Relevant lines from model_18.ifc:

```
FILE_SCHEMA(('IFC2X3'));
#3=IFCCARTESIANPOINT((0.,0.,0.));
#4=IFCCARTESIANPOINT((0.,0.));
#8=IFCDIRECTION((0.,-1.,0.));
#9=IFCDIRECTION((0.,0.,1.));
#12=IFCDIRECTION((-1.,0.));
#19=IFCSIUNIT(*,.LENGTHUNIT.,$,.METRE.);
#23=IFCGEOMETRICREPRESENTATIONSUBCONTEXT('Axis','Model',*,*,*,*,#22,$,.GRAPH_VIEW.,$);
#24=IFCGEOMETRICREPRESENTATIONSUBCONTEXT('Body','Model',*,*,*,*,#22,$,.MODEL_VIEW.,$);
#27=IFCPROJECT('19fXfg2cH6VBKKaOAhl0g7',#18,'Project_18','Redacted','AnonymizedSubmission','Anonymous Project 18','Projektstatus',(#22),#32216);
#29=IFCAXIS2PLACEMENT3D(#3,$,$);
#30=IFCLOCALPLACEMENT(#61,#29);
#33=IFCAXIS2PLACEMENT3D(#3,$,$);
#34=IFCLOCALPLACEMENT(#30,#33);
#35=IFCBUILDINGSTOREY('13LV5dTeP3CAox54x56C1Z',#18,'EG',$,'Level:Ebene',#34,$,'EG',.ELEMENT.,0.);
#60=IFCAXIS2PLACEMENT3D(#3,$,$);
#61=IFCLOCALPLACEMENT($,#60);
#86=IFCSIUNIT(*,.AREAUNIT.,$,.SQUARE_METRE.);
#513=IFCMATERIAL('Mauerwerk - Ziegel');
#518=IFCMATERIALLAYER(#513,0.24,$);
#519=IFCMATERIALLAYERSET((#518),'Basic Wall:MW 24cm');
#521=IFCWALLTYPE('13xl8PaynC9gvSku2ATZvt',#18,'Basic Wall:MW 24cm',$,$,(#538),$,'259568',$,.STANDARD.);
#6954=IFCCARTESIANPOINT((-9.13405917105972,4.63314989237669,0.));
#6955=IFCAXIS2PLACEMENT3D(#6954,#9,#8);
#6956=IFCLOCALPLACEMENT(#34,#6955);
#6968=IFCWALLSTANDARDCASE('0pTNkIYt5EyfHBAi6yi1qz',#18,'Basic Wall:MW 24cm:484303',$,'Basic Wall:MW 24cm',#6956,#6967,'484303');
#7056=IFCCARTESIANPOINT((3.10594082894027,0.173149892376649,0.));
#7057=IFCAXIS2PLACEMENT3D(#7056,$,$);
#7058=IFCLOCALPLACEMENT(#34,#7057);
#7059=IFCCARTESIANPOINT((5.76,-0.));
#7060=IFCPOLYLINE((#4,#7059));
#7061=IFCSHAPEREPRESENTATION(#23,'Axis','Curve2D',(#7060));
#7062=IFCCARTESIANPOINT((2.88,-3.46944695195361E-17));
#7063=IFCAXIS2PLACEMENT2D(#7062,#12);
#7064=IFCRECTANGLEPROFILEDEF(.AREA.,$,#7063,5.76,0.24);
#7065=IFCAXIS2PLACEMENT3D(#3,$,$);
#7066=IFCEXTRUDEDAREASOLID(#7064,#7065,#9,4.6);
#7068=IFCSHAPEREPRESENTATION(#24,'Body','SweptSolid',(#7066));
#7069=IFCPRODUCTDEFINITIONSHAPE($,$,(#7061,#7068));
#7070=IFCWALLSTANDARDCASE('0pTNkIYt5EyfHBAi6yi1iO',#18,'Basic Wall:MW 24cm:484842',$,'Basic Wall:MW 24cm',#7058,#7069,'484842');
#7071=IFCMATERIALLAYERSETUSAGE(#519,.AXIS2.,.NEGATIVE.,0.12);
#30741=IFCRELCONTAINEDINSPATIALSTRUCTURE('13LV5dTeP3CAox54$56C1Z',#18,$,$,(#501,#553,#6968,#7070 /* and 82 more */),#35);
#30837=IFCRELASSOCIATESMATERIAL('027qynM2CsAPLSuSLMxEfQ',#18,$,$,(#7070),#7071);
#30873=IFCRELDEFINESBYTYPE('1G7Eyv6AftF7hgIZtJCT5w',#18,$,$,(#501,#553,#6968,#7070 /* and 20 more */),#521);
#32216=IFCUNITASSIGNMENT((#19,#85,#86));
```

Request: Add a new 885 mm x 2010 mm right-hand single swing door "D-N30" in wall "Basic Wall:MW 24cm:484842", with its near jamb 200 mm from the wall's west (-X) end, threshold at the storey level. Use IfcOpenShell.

```python
import numpy as np
import ifcopenshell
import ifcopenshell.api.feature
import ifcopenshell.api.geometry
import ifcopenshell.api.root
import ifcopenshell.api.spatial
import ifcopenshell.api.type
import ifcopenshell.geom
import ifcopenshell.util.element
import ifcopenshell.util.placement
import ifcopenshell.util.representation
import ifcopenshell.util.shape
import ifcopenshell.util.unit

model = ifcopenshell.open("model_18.ifc")
unit_scale = ifcopenshell.util.unit.calculate_unit_scale(model)
settings = ifcopenshell.geom.settings()


def volume(element):
    """Net volume in cubic metres, openings subtracted."""
    shape = ifcopenshell.geom.create_shape(settings, element)
    return ifcopenshell.util.shape.get_volume(shape.geometry)


wall = model.by_id(7070)
storey = ifcopenshell.util.element.get_container(wall, ifc_class="IfcBuildingStorey")
context = ifcopenshell.util.representation.get_context(model, "Model", "Body", "MODEL_VIEW")
before = volume(wall)

width, height, from_end, sill = 0.885, 2.01, 0.2, 0.0  # metres

# The wall runs along its own X axis, and the end named is its -X end.
wall_shape = ifcopenshell.geom.create_shape(settings, wall)
x, y, z = ifcopenshell.util.shape.get_vertices(wall_shape.geometry).T
start = x.min() + from_end
face, thickness = float(y.min()), float(y.max() - y.min())
wall_matrix = ifcopenshell.util.placement.get_local_placement(wall.ObjectPlacement)
level = ifcopenshell.util.placement.get_local_placement(storey.ObjectPlacement)[2, 3]


def in_wall(x, y):
    """Placement at x, y metres in the wall's axes, at sill height."""
    matrix = wall_matrix.copy()
    matrix[:, 3] = wall_matrix @ np.array([x / unit_scale, y / unit_scale, 0.0, 1.0])
    matrix[2, 3] = level + sill / unit_scale
    return matrix


# Opening: a box that overshoots both wall faces by 50 mm.
opening = ifcopenshell.api.root.create_entity(model, ifc_class="IfcOpeningElement")
box = ifcopenshell.api.geometry.add_wall_representation(
    model, context=context, length=width, height=height, thickness=thickness + 0.1
)
ifcopenshell.api.geometry.assign_representation(model, product=opening, representation=box)
ifcopenshell.api.geometry.edit_object_placement(model, product=opening, matrix=in_wall(start, face - 0.05), is_si=False)
ifcopenshell.api.feature.add_feature(model, feature=opening, element=wall)

door = ifcopenshell.api.root.create_entity(model, ifc_class="IfcDoor", name="D-N30")
door.OverallWidth, door.OverallHeight = width / unit_scale, height / unit_scale
body = ifcopenshell.api.geometry.add_door_representation(
    model,
    context=context,
    overall_width=door.OverallWidth,
    overall_height=door.OverallHeight,
    operation_type="SINGLE_SWING_RIGHT",
    lining_properties={"LiningDepth": thickness / unit_scale, "ThresholdDepth": thickness / unit_scale},
)
ifcopenshell.api.geometry.assign_representation(model, product=door, representation=body)
ifcopenshell.api.spatial.assign_container(model, products=[door], relating_structure=storey)
fills = ifcopenshell.api.feature.add_filling(model, opening=opening, element=door)
fills.OwnerHistory = door.OwnerHistory  # required in IFC2X3

# IFC2X3 keeps the operation on the door style.
style = ifcopenshell.api.root.create_entity(model, ifc_class="IfcDoorStyle", name="D-N30")
style.OperationType, style.ConstructionType = "SINGLE_SWING_RIGHT", "NOTDEFINED"
style.ParameterTakesPrecedence = style.Sizeable = False
ifcopenshell.api.type.assign_type(model, related_objects=[door], relating_type=style)

# The lining spans the wall, so the door starts at the wall face.
ifcopenshell.api.geometry.edit_object_placement(model, product=door, matrix=in_wall(start, face), is_si=False)

after = volume(wall)

print(f"wall volume {before:.3f} -> {after:.3f} m3")

model.write("model_18_v2.ifc")
```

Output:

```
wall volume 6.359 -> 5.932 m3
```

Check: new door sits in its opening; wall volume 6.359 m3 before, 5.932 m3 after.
